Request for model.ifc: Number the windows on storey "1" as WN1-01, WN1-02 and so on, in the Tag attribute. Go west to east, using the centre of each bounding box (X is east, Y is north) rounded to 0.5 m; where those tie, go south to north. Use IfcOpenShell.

First a look at what the model holds.

```python
import ifcopenshell
import ifcopenshell.util.element
import ifcopenshell.util.placement

model = ifcopenshell.open("model.ifc")
print(model.schema)
storey = next(s for s in model.by_type("IfcBuildingStorey") if s.Name == "1")
windows = [e for e in ifcopenshell.util.element.get_decomposition(storey) if e.is_a("IfcWindow")]
for e in sorted(windows, key=lambda e: e.id()):
    origin = ifcopenshell.util.placement.get_local_placement(e.ObjectPlacement)[:3, 3]
    print(e.id(), e.Tag, e.Name, origin.round(2) + 0.0, sep=" | ")
```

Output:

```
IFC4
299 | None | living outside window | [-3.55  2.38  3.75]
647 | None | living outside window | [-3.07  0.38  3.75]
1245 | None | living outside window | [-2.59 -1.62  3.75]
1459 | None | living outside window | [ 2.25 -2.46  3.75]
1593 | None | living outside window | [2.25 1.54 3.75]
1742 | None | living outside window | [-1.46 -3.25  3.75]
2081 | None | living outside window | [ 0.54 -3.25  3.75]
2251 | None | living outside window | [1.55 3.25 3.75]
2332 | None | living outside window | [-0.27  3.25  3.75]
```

```python
import ifcopenshell
import ifcopenshell.geom
import ifcopenshell.util.element
import ifcopenshell.util.shape

model = ifcopenshell.open("model.ifc")
settings = ifcopenshell.geom.settings()
settings.set("use-world-coords", True)


def centre(element):
    shape = ifcopenshell.geom.create_shape(settings, element)
    return ifcopenshell.util.shape.get_bbox_centroid(shape.geometry)


storey = next(s for s in model.by_type("IfcBuildingStorey") if s.Name == "1")
windows = [e for e in ifcopenshell.util.element.get_decomposition(storey) if e.is_a("IfcWindow")]

# Insertion points can sit at a corner or the storey origin, so sort by the geometry (in metres).
centres = {e: centre(e) for e in windows}
windows.sort(key=lambda e: (round(centres[e][0] / 0.5), centres[e][1]))

for i, e in enumerate(windows, start=1):
    number = f"WN1-{i:02d}"
    e.Tag = number
    print(e.id(), number)

model.write("model_v2.ifc")
```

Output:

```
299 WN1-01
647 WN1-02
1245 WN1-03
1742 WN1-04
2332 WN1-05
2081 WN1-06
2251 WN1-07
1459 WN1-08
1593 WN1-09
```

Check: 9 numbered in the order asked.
